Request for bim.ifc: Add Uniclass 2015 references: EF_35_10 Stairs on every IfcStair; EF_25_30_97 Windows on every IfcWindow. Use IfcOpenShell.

First a look at what the model holds.

```python
import ifcopenshell

model = ifcopenshell.open("bim.ifc")
print(model.schema)
print("classifications:", [c.Name for c in model.by_type("IfcClassification")])
for ifc_class in ("IfcDoor", "IfcRoof", "IfcStair", "IfcWall", "IfcWindow"):
    print(ifc_class, len(model.by_type(ifc_class)))
```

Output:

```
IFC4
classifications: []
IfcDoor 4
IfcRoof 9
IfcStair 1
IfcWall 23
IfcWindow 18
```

```python
import ifcopenshell
import ifcopenshell.api.classification

model = ifcopenshell.open("bim.ifc")

system = ifcopenshell.api.classification.add_classification(model, classification="Uniclass 2015")

codes = {
    "IfcStair": ("EF_35_10", "Stairs"),
    "IfcWindow": ("EF_25_30_97", "Windows"),
}
for ifc_class, (code, name) in codes.items():
    products = model.by_type(ifc_class)
    ifcopenshell.api.classification.add_reference(
        model, products=products, classification=system, identification=code, name=name
    )
    print(code, len(products))

model.write("bim_v2.ifc")
```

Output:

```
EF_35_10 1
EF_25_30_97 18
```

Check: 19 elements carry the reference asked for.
